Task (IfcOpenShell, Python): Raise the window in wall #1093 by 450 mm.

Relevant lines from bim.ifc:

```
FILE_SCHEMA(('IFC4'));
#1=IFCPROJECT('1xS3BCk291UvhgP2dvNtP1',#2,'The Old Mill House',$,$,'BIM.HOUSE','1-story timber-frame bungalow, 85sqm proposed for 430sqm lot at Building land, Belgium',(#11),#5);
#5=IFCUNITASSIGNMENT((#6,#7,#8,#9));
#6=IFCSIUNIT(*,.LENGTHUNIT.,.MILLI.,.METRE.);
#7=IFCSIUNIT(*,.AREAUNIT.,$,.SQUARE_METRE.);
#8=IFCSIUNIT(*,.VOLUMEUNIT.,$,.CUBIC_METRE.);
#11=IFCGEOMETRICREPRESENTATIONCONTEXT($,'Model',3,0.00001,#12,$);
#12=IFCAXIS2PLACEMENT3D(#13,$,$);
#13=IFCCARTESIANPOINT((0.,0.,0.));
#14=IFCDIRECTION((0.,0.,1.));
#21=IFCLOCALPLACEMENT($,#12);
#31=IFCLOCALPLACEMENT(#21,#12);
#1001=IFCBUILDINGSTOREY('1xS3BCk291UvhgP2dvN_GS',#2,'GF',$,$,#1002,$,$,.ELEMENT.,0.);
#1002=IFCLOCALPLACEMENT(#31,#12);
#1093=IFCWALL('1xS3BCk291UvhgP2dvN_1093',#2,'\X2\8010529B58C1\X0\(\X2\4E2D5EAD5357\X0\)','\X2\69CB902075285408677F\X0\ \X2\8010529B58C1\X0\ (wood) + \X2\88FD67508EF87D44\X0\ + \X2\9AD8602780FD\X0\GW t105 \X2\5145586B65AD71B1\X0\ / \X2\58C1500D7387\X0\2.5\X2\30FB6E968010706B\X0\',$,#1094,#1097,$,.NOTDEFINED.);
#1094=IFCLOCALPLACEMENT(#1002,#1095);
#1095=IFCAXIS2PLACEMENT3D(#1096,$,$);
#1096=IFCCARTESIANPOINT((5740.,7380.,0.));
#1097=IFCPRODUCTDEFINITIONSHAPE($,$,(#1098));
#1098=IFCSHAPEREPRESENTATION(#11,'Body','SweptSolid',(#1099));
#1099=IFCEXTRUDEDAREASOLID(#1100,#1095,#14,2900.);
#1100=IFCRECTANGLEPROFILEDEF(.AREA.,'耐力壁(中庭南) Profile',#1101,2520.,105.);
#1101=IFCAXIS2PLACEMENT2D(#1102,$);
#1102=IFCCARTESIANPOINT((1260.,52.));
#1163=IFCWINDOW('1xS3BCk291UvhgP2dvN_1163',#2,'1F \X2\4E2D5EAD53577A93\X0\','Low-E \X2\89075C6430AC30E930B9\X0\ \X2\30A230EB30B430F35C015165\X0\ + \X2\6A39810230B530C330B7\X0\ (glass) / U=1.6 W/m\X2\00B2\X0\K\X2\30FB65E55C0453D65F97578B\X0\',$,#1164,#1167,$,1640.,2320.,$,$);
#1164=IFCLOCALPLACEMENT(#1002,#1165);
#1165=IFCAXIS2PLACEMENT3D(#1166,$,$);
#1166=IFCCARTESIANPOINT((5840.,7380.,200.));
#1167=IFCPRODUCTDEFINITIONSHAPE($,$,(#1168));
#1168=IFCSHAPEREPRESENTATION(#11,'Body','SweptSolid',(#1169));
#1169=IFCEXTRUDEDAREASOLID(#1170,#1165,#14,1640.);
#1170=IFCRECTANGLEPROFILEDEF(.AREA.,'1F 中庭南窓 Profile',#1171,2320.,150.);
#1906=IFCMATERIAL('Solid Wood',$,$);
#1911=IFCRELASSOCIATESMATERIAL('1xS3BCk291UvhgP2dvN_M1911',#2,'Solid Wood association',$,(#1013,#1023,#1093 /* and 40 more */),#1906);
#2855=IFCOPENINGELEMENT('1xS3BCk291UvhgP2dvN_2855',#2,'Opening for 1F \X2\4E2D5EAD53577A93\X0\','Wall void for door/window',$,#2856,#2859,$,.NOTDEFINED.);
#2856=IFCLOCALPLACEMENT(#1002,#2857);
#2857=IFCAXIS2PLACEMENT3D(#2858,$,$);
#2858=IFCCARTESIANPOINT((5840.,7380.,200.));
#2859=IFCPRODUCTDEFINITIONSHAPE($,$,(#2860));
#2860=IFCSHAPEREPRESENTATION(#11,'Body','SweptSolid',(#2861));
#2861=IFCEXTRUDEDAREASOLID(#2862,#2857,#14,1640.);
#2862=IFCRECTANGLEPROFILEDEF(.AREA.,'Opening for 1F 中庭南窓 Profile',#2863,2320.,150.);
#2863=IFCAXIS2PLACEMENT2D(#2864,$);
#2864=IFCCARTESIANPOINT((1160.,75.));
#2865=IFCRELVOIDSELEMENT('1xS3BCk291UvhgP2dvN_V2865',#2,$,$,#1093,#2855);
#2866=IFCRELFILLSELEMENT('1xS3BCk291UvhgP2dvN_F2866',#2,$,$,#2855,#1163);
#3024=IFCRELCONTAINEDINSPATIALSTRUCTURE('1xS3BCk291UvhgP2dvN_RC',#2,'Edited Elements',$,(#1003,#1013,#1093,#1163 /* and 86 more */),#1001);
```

```python
import numpy as np
import ifcopenshell
import ifcopenshell.api.geometry
import ifcopenshell.util.placement
import ifcopenshell.util.unit

model = ifcopenshell.open("bim.ifc")
unit_scale = ifcopenshell.util.unit.calculate_unit_scale(model)

window = model.by_guid("1xS3BCk291UvhgP2dvN_1163")
opening = window.FillsVoids[0].RelatingOpeningElement
dz = 450.0

shift = np.array([0.0, 0.0, dz])
# The window is not placed relative to its opening, so move both.
for product in (opening, window):
    matrix = ifcopenshell.util.placement.get_local_placement(product.ObjectPlacement)
    matrix[:3, 3] += shift
    ifcopenshell.api.geometry.edit_object_placement(model, product=product, matrix=matrix, is_si=False)

print(f"moved by {dz * unit_scale:+.3f} m")

model.write("bim-out.ifc")
```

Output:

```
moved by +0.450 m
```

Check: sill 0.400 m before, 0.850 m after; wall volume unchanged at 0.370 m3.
